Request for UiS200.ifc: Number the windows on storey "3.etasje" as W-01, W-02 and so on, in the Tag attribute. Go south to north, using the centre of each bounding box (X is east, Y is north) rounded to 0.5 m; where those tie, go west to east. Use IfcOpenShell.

First a look at what the model holds.

```python
import ifcopenshell
import ifcopenshell.util.element
import ifcopenshell.util.placement

model = ifcopenshell.open("UiS200.ifc")
print(model.schema)
storey = next(s for s in model.by_type("IfcBuildingStorey") if s.Name == "3.etasje")
windows = [e for e in ifcopenshell.util.element.get_decomposition(storey) if e.is_a("IfcWindow")]
for e in sorted(windows, key=lambda e: e.id()):
    origin = ifcopenshell.util.placement.get_local_placement(e.ObjectPlacement)[:3, 3]
    print(e.id(), e.Tag, e.Name, origin.round(2) + 0.0, sep=" | ")
```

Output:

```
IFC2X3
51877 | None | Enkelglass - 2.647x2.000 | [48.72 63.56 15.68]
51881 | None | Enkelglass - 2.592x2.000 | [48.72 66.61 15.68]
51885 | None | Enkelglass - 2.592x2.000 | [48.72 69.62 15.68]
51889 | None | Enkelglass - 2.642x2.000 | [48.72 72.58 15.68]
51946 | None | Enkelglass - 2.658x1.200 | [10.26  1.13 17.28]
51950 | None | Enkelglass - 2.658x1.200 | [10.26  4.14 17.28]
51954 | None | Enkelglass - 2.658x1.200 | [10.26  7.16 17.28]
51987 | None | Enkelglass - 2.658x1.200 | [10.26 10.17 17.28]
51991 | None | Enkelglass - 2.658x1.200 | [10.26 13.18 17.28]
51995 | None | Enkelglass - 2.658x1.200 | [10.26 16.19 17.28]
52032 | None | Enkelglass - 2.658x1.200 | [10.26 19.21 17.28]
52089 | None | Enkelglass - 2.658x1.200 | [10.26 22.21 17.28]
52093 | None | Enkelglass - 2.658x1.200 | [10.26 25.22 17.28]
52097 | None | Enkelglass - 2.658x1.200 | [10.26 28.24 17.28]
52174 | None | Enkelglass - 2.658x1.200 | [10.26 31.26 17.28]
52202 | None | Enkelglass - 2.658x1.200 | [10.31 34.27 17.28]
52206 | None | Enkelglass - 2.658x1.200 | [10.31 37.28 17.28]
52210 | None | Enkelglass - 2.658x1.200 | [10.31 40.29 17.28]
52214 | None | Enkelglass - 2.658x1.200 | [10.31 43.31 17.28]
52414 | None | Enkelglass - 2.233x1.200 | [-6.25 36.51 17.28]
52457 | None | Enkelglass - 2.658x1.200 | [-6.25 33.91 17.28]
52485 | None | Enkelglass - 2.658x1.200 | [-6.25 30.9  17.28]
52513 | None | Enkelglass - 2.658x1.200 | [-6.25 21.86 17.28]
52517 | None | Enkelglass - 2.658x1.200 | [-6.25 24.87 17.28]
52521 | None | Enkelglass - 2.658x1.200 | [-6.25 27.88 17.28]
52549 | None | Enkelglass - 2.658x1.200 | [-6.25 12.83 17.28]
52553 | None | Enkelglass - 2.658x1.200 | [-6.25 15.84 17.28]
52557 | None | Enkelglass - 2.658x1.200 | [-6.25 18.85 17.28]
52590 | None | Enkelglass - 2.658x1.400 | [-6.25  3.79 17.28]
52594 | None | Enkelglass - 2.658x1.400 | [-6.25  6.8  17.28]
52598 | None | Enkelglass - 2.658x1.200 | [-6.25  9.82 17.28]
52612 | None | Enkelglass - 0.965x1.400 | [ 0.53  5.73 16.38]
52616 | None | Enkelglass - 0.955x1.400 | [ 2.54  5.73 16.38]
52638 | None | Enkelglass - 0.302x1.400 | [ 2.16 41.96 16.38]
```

```python
import ifcopenshell
import ifcopenshell.geom
import ifcopenshell.util.element
import ifcopenshell.util.shape

model = ifcopenshell.open("UiS200.ifc")
settings = ifcopenshell.geom.settings()
settings.set("use-world-coords", True)


def centre(element):
    shape = ifcopenshell.geom.create_shape(settings, element)
    return ifcopenshell.util.shape.get_bbox_centroid(shape.geometry)


storey = next(s for s in model.by_type("IfcBuildingStorey") if s.Name == "3.etasje")
windows = [e for e in ifcopenshell.util.element.get_decomposition(storey) if e.is_a("IfcWindow")]

# Insertion points can sit at a corner or the storey origin, so sort by the geometry (in metres).
centres = {e: centre(e) for e in windows}
windows.sort(key=lambda e: (round(centres[e][1] / 0.5), centres[e][0]))

for i, e in enumerate(windows, start=1):
    number = f"W-{i:02d}"
    e.Tag = number
    print(e.id(), number)

model.write("UiS200_edited.ifc")
```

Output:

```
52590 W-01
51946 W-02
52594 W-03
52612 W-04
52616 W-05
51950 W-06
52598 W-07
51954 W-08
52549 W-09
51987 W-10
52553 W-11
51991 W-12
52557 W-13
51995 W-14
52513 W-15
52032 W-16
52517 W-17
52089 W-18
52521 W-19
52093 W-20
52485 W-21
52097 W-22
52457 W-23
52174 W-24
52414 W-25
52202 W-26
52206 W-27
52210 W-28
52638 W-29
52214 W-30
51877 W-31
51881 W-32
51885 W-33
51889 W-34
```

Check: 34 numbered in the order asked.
